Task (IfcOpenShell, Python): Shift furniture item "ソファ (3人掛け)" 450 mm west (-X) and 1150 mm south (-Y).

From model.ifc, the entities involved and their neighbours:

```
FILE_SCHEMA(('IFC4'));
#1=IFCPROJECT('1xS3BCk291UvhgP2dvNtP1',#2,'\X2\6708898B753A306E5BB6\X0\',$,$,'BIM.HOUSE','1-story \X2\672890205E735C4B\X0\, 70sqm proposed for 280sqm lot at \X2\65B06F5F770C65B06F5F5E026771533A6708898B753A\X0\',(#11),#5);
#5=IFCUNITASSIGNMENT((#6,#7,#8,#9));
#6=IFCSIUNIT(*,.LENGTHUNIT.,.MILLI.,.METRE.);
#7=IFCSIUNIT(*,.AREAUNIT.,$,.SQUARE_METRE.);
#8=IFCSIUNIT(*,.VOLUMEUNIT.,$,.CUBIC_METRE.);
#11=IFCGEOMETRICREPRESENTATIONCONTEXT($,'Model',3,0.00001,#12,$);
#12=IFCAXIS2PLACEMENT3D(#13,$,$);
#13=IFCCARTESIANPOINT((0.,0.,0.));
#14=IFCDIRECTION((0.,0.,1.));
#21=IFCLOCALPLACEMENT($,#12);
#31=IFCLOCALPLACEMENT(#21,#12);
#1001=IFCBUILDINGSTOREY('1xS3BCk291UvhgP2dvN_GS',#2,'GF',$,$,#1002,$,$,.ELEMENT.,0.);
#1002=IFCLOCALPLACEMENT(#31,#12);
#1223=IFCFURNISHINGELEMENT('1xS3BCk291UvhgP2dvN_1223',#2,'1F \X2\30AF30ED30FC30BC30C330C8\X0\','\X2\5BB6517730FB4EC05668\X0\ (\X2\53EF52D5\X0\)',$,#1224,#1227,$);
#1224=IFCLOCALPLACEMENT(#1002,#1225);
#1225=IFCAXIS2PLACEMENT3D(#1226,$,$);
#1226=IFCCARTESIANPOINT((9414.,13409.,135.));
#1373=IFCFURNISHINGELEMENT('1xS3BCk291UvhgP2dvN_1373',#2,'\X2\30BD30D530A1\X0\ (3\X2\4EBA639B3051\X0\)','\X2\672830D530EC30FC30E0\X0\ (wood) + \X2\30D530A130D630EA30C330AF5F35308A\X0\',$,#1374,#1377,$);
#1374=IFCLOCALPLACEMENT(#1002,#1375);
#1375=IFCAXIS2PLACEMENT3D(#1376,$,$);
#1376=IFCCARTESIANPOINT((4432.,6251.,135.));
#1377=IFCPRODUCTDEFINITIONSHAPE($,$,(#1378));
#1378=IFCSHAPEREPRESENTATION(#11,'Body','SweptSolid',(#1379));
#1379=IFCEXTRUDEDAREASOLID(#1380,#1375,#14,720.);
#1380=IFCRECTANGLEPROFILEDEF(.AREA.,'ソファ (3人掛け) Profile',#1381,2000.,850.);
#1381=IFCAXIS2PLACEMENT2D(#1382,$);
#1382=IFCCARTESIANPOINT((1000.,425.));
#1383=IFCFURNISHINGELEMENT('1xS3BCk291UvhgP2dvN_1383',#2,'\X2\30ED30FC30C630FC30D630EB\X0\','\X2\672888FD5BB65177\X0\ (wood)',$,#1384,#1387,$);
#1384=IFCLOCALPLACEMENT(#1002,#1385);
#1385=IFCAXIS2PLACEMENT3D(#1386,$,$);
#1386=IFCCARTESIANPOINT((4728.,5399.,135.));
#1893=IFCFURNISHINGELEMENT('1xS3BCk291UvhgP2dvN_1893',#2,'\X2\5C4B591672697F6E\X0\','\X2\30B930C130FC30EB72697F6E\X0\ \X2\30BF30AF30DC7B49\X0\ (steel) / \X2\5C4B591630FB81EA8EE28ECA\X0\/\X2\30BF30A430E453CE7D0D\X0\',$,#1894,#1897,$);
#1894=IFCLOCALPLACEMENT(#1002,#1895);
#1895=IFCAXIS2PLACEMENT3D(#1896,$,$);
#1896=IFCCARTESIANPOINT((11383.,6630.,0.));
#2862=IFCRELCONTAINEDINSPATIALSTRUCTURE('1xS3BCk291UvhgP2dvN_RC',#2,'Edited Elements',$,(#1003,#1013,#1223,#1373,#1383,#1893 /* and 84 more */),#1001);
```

```python
import ifcopenshell
import ifcopenshell.api.geometry
import ifcopenshell.util.placement

model = ifcopenshell.open("model.ifc")

item = model.by_guid("1xS3BCk291UvhgP2dvN_1373")
matrix = ifcopenshell.util.placement.get_local_placement(item.ObjectPlacement)
matrix[0, 3] -= 450.0
matrix[1, 3] -= 1150.0
ifcopenshell.api.geometry.edit_object_placement(model, product=item, matrix=matrix, is_si=False)

print(ifcopenshell.util.placement.get_local_placement(item.ObjectPlacement).round(3) + 0.0)

model.write("model-out.ifc")
```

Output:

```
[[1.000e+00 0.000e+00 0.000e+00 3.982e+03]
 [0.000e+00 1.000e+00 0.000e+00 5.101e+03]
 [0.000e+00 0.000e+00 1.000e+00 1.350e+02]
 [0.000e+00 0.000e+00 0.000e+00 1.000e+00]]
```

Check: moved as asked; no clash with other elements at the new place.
